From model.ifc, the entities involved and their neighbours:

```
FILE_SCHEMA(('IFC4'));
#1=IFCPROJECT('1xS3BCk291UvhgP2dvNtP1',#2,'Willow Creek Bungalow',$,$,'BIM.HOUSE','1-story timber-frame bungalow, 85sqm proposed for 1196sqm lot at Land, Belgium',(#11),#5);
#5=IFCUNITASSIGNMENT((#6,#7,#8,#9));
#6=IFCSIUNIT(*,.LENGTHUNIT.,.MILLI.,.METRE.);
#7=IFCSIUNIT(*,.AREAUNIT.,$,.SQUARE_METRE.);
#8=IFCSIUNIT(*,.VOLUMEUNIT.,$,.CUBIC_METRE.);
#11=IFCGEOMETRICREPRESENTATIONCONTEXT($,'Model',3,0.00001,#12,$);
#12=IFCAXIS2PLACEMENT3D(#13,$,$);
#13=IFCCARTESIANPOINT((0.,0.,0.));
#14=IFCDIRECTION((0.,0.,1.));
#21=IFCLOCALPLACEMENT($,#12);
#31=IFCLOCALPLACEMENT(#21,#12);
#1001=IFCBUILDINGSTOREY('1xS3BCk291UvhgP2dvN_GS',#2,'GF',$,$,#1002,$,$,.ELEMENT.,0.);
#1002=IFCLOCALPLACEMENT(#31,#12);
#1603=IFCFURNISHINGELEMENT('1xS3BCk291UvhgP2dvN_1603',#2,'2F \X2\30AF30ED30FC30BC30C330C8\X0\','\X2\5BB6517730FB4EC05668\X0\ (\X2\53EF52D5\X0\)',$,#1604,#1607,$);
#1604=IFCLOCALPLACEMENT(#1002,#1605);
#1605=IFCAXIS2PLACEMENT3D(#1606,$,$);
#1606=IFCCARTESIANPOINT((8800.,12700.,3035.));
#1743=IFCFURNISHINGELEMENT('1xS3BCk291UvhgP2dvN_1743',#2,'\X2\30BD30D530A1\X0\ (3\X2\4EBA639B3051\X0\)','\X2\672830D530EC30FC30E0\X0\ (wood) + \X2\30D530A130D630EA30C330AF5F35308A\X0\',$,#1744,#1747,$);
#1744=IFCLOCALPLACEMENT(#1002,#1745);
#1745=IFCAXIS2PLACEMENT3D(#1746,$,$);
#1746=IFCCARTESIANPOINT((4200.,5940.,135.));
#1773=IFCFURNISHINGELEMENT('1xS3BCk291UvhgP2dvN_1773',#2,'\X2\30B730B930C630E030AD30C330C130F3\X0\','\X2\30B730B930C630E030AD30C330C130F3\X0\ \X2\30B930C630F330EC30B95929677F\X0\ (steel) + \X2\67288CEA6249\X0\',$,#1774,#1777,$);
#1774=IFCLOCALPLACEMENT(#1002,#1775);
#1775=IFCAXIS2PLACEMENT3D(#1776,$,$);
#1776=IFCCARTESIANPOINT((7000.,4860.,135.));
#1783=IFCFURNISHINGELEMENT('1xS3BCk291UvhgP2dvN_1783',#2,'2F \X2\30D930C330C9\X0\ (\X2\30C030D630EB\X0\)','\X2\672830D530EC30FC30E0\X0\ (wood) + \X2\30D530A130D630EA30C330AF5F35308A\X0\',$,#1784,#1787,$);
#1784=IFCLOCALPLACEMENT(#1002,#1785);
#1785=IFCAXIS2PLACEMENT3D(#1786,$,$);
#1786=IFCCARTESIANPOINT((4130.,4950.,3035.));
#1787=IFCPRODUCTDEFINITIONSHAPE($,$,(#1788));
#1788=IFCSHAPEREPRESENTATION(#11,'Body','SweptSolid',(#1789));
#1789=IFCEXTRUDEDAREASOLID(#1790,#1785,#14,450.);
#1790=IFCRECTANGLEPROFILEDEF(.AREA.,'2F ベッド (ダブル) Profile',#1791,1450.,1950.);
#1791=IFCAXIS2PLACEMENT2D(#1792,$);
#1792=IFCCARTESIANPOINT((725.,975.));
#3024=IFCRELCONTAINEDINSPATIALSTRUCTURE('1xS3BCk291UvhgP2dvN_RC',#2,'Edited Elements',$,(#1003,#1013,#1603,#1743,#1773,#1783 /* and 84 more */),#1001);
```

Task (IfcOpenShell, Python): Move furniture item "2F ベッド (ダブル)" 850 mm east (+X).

```python
import ifcopenshell
import ifcopenshell.api.geometry
import ifcopenshell.util.placement

model = ifcopenshell.open("model.ifc")

item = model.by_id(1783)
matrix = ifcopenshell.util.placement.get_local_placement(item.ObjectPlacement)
matrix[0, 3] += 850.0
ifcopenshell.api.geometry.edit_object_placement(model, product=item, matrix=matrix, is_si=False)

print(ifcopenshell.util.placement.get_local_placement(item.ObjectPlacement).round(3) + 0.0)

model.write("model_rev.ifc")
```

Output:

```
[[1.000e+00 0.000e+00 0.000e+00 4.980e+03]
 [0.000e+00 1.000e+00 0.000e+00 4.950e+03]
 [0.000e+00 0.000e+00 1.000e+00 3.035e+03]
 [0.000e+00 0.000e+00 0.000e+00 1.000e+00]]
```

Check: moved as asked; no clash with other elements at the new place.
